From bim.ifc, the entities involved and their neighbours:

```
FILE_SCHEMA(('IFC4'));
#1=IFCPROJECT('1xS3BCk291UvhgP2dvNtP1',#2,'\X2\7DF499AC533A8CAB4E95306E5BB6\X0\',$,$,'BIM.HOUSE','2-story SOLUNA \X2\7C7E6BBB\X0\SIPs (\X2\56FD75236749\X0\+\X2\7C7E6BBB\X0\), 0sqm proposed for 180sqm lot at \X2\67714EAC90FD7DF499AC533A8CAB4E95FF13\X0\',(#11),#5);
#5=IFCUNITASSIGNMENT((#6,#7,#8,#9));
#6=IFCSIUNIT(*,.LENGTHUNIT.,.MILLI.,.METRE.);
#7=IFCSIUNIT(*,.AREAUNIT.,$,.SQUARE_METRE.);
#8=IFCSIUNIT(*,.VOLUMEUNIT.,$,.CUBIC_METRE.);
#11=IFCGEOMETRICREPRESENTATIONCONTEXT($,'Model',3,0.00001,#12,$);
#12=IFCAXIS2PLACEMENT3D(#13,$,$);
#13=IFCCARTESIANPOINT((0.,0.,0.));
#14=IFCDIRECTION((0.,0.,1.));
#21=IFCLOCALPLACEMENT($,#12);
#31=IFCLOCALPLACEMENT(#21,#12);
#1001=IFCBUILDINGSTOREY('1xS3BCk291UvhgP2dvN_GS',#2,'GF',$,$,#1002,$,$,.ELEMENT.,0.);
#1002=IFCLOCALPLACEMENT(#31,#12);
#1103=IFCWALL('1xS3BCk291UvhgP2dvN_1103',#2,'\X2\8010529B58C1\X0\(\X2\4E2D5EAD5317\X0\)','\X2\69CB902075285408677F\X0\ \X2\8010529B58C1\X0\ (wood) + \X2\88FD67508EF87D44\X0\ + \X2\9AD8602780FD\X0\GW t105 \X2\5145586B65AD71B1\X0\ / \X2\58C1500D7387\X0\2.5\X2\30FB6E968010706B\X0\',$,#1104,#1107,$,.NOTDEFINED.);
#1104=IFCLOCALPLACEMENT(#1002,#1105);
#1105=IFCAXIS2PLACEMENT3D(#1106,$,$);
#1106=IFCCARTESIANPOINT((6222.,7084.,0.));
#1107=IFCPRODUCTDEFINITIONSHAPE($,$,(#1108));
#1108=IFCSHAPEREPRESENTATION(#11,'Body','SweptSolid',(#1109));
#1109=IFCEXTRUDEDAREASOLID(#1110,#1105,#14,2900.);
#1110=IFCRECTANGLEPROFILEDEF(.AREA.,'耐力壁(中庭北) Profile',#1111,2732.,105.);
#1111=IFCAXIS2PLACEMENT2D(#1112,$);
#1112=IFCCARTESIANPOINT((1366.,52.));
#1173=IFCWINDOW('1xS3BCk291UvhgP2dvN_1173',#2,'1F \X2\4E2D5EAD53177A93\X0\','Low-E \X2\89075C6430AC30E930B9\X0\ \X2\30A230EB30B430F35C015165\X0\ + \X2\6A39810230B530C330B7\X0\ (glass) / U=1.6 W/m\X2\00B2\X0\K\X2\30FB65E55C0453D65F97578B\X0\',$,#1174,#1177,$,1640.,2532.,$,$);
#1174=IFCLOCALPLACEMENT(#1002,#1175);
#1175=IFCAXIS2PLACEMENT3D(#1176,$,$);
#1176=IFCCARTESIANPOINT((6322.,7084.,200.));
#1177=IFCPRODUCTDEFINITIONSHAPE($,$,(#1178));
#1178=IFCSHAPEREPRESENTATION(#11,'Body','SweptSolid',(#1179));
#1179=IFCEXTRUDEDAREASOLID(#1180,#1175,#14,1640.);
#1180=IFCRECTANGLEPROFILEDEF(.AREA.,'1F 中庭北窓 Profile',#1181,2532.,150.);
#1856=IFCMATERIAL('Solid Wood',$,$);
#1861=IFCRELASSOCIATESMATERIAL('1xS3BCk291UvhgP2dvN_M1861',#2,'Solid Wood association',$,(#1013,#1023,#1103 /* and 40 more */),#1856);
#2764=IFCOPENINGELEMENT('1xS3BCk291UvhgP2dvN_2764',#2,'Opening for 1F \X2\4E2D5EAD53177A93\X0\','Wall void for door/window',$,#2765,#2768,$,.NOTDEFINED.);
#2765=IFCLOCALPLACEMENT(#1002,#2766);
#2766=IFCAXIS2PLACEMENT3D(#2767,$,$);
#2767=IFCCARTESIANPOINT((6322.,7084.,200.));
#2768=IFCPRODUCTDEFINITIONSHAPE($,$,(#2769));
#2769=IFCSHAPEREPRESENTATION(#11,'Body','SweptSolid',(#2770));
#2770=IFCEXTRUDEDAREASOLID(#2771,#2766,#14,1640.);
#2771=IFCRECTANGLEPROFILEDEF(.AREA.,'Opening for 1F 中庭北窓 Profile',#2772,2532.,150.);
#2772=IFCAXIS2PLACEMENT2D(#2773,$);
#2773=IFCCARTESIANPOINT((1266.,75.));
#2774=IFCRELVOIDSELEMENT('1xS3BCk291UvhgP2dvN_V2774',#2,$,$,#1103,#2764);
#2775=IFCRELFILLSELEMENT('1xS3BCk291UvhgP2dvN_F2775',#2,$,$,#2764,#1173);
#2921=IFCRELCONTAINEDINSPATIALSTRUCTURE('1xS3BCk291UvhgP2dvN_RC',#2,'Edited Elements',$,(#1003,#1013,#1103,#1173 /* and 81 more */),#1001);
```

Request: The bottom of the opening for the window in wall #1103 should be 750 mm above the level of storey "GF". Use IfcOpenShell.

```python
import numpy as np
import ifcopenshell
import ifcopenshell.api.geometry
import ifcopenshell.geom
import ifcopenshell.util.element
import ifcopenshell.util.placement
import ifcopenshell.util.shape
import ifcopenshell.util.unit

model = ifcopenshell.open("bim.ifc")
unit_scale = ifcopenshell.util.unit.calculate_unit_scale(model)

window = model.by_id(1173)
opening = window.FillsVoids[0].RelatingOpeningElement
storey = ifcopenshell.util.element.get_container(window, ifc_class="IfcBuildingStorey")
level = ifcopenshell.util.placement.get_local_placement(storey.ObjectPlacement)[2, 3]

# The opening's origin need not be at the sill, so measure its lowest point.
shape = ifcopenshell.geom.create_shape(ifcopenshell.geom.settings(), opening)
bottom = ifcopenshell.util.shape.get_shape_bottom_elevation(shape, shape.geometry) / unit_scale
dz = level + 0.75 / unit_scale - bottom

shift = np.array([0.0, 0.0, dz])
# The window is not placed relative to its opening, so move both.
for product in (opening, window):
    matrix = ifcopenshell.util.placement.get_local_placement(product.ObjectPlacement)
    matrix[:3, 3] += shift
    ifcopenshell.api.geometry.edit_object_placement(model, product=product, matrix=matrix, is_si=False)

print(f"moved by {dz * unit_scale:+.3f} m")

model.write("bim_rev.ifc")
```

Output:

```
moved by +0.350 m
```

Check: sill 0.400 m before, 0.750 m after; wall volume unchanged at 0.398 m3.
